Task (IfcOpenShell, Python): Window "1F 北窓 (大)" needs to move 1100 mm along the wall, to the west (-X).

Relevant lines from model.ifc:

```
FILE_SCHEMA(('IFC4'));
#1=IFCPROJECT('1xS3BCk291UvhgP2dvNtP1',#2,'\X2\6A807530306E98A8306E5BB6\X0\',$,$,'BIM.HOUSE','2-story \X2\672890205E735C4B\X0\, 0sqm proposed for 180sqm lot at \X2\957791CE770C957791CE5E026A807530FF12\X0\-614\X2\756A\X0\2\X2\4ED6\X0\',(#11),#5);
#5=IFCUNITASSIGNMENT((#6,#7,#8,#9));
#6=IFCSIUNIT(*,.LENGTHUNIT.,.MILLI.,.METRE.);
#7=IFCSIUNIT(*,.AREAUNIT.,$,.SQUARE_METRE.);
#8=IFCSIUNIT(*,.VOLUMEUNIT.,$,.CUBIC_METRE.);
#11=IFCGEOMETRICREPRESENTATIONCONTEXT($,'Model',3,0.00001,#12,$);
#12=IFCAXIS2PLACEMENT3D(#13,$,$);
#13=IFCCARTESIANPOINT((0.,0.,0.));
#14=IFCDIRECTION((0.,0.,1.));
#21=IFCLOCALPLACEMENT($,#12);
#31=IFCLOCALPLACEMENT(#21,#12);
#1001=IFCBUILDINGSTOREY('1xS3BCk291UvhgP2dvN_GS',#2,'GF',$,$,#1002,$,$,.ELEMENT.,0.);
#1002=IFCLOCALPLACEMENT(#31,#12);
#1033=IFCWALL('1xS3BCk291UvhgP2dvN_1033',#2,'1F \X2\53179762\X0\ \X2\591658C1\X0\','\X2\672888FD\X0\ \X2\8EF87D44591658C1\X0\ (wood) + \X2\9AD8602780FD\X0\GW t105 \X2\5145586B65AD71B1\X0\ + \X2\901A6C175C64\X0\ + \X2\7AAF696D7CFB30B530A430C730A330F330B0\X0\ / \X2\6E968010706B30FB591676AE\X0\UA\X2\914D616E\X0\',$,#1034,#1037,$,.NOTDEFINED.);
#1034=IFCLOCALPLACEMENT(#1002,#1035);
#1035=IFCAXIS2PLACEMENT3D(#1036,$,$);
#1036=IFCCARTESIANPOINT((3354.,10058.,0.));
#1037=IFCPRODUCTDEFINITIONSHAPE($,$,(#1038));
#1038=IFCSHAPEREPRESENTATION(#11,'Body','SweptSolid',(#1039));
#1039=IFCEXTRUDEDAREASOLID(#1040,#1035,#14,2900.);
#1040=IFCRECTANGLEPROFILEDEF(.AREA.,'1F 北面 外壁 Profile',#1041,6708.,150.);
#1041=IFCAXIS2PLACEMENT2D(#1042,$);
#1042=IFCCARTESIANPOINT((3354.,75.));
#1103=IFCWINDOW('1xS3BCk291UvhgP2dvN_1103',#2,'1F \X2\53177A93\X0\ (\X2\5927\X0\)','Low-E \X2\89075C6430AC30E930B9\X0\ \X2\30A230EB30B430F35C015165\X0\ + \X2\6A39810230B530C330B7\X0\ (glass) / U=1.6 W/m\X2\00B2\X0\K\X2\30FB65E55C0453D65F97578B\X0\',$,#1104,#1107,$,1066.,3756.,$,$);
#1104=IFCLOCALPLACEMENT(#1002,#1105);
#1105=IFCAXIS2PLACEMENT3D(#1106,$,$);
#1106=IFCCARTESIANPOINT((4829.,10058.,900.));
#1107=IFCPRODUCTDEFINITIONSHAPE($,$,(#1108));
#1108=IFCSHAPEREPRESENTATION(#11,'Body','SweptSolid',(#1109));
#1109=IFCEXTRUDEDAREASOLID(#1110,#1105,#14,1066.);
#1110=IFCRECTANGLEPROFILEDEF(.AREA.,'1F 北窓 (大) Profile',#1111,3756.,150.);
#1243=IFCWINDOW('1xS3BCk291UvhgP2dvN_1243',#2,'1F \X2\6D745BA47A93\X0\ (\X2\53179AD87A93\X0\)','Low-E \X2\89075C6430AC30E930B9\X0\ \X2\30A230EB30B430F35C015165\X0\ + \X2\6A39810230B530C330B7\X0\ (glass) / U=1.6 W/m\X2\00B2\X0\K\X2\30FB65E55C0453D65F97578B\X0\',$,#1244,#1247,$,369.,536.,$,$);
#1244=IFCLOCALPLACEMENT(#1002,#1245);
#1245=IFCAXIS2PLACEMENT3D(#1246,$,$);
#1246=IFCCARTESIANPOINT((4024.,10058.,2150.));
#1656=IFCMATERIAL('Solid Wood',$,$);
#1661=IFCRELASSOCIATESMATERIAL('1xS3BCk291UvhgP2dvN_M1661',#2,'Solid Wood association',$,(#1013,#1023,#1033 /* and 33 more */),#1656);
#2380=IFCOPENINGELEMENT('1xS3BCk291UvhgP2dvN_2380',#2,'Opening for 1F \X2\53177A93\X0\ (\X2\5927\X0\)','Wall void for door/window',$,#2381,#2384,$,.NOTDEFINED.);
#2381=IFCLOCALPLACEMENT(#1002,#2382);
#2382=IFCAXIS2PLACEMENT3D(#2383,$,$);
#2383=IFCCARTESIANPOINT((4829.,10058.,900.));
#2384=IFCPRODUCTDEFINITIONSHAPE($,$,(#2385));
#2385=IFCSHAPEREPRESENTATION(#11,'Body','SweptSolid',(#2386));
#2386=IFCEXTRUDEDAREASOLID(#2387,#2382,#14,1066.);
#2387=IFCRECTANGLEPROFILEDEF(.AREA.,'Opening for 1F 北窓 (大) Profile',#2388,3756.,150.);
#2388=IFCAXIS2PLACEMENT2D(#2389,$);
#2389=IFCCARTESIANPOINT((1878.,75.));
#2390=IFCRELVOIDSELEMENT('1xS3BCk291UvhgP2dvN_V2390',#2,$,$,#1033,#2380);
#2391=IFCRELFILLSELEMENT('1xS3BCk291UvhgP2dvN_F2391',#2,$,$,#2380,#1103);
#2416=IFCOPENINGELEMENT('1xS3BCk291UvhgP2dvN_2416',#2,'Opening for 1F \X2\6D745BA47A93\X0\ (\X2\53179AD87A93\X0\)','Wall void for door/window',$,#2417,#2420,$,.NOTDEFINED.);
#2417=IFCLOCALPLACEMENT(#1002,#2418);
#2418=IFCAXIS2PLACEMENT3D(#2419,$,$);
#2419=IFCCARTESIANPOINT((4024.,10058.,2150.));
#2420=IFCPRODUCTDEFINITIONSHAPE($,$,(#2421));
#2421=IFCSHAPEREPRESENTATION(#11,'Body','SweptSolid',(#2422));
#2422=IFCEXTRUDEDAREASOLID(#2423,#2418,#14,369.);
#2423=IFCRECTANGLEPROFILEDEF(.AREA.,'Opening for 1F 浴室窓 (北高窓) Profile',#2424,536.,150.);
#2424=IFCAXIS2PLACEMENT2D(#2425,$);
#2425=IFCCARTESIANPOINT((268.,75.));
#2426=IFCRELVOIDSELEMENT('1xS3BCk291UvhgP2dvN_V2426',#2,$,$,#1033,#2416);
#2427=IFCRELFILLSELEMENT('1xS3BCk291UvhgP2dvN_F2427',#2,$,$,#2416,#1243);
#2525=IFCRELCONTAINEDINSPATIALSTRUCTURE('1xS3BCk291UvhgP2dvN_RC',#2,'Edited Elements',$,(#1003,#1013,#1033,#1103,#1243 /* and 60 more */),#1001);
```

```python
import ifcopenshell
import ifcopenshell.api.geometry
import ifcopenshell.util.placement
import ifcopenshell.util.unit

model = ifcopenshell.open("model.ifc")
unit_scale = ifcopenshell.util.unit.calculate_unit_scale(model)

window = model.by_guid("1xS3BCk291UvhgP2dvN_1103")
opening = window.FillsVoids[0].RelatingOpeningElement
wall = opening.VoidsElements[0].RelatingBuildingElement

wall_matrix = ifcopenshell.util.placement.get_local_placement(wall.ObjectPlacement)
shift = wall_matrix[:3, 0] * -1.1 / unit_scale
before = ifcopenshell.util.placement.get_local_placement(window.ObjectPlacement)[:3, 3].copy()

# The window is not placed relative to its opening, so move both.
for product in (opening, window):
    matrix = ifcopenshell.util.placement.get_local_placement(product.ObjectPlacement)
    matrix[:3, 3] += shift
    ifcopenshell.api.geometry.edit_object_placement(model, product=product, matrix=matrix, is_si=False)

after = ifcopenshell.util.placement.get_local_placement(window.ObjectPlacement)[:3, 3]
print("window moved by", (after - before).round(3) + 0.0)

model.write("model-out.ifc")
```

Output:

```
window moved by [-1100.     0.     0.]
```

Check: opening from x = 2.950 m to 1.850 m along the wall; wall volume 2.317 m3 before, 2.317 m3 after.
